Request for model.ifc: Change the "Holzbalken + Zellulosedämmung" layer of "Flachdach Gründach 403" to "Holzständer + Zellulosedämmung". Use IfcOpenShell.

First a look at what the model holds.

```python
import ifcopenshell
import ifcopenshell.util.element

model = ifcopenshell.open("model.ifc")
print(model.schema)
for layer_set in model.by_type("IfcMaterialLayerSet"):
    if layer_set.LayerSetName == "Flachdach Gründach 403":
        for layer in layer_set.MaterialLayers:
            print(layer.id(), layer.Material and layer.Material.Name, layer.LayerThickness, sep=" | ")
        print(len(ifcopenshell.util.element.get_elements_by_material(model, layer_set)), "elements and types use it")
print(sorted(m.Name for m in model.by_type("IfcMaterial") if m.Name)[:60])
```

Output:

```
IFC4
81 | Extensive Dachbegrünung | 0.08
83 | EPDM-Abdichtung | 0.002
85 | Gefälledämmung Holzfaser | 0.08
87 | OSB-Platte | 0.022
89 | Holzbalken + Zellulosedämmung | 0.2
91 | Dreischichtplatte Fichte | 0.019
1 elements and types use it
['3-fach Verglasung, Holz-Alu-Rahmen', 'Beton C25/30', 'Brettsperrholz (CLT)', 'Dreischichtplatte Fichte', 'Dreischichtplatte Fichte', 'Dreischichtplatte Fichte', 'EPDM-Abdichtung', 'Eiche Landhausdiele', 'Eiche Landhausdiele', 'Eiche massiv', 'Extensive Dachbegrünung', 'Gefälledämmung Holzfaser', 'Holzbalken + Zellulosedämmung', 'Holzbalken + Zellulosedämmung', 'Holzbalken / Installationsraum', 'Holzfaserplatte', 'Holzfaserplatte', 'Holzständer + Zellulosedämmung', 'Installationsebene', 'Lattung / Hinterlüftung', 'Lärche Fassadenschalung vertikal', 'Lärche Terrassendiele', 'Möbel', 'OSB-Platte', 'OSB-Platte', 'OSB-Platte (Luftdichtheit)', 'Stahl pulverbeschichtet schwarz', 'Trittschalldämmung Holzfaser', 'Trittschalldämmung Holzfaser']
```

```python
import ifcopenshell
import ifcopenshell.api.material

model = ifcopenshell.open("model.ifc")

layer_set = next(s for s in model.by_type("IfcMaterialLayerSet") if s.LayerSetName == "Flachdach Gründach 403")
layer = next(l for l in layer_set.MaterialLayers if l.Material and l.Material.Name == "Holzbalken + Zellulosedämmung")
material = next(m for m in model.by_type("IfcMaterial") if m.Name == "Holzständer + Zellulosedämmung")

# Point this one layer at the other material; renaming the old one would change it everywhere.
ifcopenshell.api.material.edit_layer(model, layer=layer, attributes={"Name": material.Name}, material=material)

print([l.Material.Name if l.Material else None for l in layer_set.MaterialLayers])

model.write("model_v2.ifc")
```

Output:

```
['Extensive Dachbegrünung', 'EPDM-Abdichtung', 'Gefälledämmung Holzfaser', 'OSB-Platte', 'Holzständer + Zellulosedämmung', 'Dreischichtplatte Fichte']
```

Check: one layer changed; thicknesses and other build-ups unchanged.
